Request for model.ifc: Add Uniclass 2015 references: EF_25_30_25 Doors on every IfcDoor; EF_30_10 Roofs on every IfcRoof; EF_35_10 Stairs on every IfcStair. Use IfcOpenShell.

First a look at what the model holds.

```python
import ifcopenshell

model = ifcopenshell.open("model.ifc")
print(model.schema)
print("classifications:", [c.Name for c in model.by_type("IfcClassification")])
for ifc_class in ("IfcDoor", "IfcRoof", "IfcStair", "IfcWall", "IfcWindow"):
    print(ifc_class, len(model.by_type(ifc_class)))
```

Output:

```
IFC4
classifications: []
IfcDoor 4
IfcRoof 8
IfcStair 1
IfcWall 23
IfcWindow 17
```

```python
import ifcopenshell
import ifcopenshell.api.classification

model = ifcopenshell.open("model.ifc")

system = ifcopenshell.api.classification.add_classification(model, classification="Uniclass 2015")

codes = {
    "IfcDoor": ("EF_25_30_25", "Doors"),
    "IfcRoof": ("EF_30_10", "Roofs"),
    "IfcStair": ("EF_35_10", "Stairs"),
}
for ifc_class, (code, name) in codes.items():
    products = model.by_type(ifc_class)
    ifcopenshell.api.classification.add_reference(
        model, products=products, classification=system, identification=code, name=name
    )
    print(code, len(products))

model.write("model_edited.ifc")
```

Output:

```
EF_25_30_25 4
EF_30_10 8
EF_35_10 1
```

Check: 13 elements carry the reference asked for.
